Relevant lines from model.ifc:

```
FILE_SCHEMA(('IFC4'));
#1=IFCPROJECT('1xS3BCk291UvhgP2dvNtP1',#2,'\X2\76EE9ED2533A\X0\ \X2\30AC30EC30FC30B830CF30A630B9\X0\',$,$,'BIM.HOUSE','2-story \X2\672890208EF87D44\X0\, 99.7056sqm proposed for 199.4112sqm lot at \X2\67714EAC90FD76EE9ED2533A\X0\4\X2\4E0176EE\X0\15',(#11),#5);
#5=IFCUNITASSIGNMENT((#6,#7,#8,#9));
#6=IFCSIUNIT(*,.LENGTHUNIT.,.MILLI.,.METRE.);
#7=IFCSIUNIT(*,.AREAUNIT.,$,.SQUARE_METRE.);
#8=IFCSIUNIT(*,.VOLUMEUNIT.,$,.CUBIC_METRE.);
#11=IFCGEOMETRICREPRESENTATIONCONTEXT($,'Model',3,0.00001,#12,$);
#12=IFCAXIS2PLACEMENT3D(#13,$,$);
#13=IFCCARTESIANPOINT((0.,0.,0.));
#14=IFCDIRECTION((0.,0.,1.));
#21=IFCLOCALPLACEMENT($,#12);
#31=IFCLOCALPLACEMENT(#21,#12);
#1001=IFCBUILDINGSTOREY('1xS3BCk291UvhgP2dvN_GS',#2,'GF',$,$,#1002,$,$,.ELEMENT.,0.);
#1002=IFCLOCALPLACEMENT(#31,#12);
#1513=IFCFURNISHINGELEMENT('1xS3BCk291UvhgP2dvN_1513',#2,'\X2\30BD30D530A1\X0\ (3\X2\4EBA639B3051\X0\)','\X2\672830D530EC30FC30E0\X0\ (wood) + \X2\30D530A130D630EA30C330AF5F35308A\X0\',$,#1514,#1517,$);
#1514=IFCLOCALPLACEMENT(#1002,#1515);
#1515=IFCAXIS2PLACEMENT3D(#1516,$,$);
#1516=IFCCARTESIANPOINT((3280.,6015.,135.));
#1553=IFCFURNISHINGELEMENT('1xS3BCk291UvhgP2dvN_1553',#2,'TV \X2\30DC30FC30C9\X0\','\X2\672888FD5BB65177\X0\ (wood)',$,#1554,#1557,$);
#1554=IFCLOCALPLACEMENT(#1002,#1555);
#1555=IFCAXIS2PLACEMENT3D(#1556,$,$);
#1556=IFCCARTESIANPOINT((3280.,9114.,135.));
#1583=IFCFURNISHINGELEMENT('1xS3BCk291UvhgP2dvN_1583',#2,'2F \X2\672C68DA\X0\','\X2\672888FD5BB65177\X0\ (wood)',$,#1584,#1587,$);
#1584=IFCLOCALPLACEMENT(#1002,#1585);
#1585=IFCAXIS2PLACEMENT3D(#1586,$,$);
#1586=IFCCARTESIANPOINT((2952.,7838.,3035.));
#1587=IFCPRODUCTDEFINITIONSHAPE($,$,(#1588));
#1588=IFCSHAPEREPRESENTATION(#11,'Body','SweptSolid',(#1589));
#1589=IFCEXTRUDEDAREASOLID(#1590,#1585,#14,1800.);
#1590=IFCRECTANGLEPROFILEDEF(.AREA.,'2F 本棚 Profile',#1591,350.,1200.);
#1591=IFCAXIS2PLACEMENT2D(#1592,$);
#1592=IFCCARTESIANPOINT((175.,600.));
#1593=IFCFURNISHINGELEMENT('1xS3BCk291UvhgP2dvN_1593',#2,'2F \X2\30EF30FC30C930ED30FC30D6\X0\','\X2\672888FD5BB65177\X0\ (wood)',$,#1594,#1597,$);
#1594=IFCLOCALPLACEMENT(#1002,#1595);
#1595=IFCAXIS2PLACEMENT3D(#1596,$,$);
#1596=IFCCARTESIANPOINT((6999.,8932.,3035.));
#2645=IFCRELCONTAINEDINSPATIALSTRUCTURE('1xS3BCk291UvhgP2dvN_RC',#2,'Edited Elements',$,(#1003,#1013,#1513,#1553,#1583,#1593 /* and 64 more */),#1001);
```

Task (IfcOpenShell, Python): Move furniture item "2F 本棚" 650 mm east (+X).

```python
import ifcopenshell
import ifcopenshell.api.geometry
import ifcopenshell.util.placement
import ifcopenshell.util.unit

model = ifcopenshell.open("model.ifc")
unit_scale = ifcopenshell.util.unit.calculate_unit_scale(model)

item = model.by_id(1583)
matrix = ifcopenshell.util.placement.get_local_placement(item.ObjectPlacement)
matrix[0, 3] += 0.65 / unit_scale
ifcopenshell.api.geometry.edit_object_placement(model, product=item, matrix=matrix, is_si=False)

print(ifcopenshell.util.placement.get_local_placement(item.ObjectPlacement).round(3) + 0.0)

model.write("model_v2.ifc")
```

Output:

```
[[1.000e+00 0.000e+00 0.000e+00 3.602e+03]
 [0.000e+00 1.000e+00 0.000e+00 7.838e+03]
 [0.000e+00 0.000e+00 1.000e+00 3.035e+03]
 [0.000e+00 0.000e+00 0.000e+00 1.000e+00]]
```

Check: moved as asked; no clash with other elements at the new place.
